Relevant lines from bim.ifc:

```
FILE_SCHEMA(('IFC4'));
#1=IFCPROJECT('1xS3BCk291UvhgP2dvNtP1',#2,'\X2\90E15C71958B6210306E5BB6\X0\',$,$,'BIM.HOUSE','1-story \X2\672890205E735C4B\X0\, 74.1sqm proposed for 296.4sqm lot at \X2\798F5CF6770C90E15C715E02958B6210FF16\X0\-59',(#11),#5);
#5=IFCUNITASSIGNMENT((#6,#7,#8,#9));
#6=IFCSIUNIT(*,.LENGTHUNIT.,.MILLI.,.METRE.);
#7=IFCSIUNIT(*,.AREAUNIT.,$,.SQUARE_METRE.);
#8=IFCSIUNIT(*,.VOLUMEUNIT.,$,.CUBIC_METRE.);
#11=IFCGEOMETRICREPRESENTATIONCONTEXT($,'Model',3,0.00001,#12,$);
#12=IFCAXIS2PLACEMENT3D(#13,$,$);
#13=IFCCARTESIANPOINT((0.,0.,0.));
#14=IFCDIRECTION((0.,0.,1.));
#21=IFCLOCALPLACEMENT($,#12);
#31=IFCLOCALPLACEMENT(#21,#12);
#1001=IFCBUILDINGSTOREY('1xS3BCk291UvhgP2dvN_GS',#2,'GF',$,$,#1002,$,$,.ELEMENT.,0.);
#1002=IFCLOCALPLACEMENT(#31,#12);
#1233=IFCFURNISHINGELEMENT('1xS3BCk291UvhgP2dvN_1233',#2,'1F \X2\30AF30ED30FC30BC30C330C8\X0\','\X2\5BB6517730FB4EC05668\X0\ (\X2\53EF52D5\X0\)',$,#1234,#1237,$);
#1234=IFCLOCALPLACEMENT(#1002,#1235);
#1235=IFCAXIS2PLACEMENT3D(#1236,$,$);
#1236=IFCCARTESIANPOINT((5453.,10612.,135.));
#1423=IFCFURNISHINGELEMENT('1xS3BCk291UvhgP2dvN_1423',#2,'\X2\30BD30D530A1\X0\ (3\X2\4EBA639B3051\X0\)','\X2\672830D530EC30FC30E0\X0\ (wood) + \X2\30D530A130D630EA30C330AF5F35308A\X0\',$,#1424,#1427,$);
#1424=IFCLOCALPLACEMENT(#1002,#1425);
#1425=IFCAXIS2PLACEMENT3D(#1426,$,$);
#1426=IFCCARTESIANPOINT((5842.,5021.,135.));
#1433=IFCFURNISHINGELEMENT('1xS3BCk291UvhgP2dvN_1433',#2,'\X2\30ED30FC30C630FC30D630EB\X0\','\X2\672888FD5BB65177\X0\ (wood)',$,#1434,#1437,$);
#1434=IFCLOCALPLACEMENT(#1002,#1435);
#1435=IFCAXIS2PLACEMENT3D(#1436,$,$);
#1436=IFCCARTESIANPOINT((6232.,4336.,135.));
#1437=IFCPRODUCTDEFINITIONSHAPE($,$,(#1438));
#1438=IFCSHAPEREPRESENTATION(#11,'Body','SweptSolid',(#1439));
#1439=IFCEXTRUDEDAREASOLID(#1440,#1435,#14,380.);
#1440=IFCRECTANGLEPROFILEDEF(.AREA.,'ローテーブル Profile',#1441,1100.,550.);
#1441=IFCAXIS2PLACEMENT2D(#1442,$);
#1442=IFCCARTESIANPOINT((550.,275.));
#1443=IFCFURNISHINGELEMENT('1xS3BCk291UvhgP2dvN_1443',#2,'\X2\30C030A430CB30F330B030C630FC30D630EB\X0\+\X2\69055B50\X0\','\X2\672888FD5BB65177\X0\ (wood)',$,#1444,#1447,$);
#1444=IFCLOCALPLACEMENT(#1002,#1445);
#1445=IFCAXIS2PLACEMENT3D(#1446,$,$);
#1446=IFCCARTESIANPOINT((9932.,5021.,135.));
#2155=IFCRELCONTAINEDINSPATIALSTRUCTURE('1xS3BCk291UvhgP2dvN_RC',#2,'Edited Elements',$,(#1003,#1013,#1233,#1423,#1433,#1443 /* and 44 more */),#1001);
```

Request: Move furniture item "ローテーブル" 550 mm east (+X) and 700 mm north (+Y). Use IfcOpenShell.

```python
import ifcopenshell
import ifcopenshell.api.geometry
import ifcopenshell.util.placement
import ifcopenshell.util.unit

model = ifcopenshell.open("bim.ifc")
unit_scale = ifcopenshell.util.unit.calculate_unit_scale(model)

item = model.by_guid("1xS3BCk291UvhgP2dvN_1433")
matrix = ifcopenshell.util.placement.get_local_placement(item.ObjectPlacement)
matrix[0, 3] += 0.55 / unit_scale
matrix[1, 3] += 0.7 / unit_scale
ifcopenshell.api.geometry.edit_object_placement(model, product=item, matrix=matrix, is_si=False)

print(ifcopenshell.util.placement.get_local_placement(item.ObjectPlacement).round(3) + 0.0)

model.write("bim_edited.ifc")
```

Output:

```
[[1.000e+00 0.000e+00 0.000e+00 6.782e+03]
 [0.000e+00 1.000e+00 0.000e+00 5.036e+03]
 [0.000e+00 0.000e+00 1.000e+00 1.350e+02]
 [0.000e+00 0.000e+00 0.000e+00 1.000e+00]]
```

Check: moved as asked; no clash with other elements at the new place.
